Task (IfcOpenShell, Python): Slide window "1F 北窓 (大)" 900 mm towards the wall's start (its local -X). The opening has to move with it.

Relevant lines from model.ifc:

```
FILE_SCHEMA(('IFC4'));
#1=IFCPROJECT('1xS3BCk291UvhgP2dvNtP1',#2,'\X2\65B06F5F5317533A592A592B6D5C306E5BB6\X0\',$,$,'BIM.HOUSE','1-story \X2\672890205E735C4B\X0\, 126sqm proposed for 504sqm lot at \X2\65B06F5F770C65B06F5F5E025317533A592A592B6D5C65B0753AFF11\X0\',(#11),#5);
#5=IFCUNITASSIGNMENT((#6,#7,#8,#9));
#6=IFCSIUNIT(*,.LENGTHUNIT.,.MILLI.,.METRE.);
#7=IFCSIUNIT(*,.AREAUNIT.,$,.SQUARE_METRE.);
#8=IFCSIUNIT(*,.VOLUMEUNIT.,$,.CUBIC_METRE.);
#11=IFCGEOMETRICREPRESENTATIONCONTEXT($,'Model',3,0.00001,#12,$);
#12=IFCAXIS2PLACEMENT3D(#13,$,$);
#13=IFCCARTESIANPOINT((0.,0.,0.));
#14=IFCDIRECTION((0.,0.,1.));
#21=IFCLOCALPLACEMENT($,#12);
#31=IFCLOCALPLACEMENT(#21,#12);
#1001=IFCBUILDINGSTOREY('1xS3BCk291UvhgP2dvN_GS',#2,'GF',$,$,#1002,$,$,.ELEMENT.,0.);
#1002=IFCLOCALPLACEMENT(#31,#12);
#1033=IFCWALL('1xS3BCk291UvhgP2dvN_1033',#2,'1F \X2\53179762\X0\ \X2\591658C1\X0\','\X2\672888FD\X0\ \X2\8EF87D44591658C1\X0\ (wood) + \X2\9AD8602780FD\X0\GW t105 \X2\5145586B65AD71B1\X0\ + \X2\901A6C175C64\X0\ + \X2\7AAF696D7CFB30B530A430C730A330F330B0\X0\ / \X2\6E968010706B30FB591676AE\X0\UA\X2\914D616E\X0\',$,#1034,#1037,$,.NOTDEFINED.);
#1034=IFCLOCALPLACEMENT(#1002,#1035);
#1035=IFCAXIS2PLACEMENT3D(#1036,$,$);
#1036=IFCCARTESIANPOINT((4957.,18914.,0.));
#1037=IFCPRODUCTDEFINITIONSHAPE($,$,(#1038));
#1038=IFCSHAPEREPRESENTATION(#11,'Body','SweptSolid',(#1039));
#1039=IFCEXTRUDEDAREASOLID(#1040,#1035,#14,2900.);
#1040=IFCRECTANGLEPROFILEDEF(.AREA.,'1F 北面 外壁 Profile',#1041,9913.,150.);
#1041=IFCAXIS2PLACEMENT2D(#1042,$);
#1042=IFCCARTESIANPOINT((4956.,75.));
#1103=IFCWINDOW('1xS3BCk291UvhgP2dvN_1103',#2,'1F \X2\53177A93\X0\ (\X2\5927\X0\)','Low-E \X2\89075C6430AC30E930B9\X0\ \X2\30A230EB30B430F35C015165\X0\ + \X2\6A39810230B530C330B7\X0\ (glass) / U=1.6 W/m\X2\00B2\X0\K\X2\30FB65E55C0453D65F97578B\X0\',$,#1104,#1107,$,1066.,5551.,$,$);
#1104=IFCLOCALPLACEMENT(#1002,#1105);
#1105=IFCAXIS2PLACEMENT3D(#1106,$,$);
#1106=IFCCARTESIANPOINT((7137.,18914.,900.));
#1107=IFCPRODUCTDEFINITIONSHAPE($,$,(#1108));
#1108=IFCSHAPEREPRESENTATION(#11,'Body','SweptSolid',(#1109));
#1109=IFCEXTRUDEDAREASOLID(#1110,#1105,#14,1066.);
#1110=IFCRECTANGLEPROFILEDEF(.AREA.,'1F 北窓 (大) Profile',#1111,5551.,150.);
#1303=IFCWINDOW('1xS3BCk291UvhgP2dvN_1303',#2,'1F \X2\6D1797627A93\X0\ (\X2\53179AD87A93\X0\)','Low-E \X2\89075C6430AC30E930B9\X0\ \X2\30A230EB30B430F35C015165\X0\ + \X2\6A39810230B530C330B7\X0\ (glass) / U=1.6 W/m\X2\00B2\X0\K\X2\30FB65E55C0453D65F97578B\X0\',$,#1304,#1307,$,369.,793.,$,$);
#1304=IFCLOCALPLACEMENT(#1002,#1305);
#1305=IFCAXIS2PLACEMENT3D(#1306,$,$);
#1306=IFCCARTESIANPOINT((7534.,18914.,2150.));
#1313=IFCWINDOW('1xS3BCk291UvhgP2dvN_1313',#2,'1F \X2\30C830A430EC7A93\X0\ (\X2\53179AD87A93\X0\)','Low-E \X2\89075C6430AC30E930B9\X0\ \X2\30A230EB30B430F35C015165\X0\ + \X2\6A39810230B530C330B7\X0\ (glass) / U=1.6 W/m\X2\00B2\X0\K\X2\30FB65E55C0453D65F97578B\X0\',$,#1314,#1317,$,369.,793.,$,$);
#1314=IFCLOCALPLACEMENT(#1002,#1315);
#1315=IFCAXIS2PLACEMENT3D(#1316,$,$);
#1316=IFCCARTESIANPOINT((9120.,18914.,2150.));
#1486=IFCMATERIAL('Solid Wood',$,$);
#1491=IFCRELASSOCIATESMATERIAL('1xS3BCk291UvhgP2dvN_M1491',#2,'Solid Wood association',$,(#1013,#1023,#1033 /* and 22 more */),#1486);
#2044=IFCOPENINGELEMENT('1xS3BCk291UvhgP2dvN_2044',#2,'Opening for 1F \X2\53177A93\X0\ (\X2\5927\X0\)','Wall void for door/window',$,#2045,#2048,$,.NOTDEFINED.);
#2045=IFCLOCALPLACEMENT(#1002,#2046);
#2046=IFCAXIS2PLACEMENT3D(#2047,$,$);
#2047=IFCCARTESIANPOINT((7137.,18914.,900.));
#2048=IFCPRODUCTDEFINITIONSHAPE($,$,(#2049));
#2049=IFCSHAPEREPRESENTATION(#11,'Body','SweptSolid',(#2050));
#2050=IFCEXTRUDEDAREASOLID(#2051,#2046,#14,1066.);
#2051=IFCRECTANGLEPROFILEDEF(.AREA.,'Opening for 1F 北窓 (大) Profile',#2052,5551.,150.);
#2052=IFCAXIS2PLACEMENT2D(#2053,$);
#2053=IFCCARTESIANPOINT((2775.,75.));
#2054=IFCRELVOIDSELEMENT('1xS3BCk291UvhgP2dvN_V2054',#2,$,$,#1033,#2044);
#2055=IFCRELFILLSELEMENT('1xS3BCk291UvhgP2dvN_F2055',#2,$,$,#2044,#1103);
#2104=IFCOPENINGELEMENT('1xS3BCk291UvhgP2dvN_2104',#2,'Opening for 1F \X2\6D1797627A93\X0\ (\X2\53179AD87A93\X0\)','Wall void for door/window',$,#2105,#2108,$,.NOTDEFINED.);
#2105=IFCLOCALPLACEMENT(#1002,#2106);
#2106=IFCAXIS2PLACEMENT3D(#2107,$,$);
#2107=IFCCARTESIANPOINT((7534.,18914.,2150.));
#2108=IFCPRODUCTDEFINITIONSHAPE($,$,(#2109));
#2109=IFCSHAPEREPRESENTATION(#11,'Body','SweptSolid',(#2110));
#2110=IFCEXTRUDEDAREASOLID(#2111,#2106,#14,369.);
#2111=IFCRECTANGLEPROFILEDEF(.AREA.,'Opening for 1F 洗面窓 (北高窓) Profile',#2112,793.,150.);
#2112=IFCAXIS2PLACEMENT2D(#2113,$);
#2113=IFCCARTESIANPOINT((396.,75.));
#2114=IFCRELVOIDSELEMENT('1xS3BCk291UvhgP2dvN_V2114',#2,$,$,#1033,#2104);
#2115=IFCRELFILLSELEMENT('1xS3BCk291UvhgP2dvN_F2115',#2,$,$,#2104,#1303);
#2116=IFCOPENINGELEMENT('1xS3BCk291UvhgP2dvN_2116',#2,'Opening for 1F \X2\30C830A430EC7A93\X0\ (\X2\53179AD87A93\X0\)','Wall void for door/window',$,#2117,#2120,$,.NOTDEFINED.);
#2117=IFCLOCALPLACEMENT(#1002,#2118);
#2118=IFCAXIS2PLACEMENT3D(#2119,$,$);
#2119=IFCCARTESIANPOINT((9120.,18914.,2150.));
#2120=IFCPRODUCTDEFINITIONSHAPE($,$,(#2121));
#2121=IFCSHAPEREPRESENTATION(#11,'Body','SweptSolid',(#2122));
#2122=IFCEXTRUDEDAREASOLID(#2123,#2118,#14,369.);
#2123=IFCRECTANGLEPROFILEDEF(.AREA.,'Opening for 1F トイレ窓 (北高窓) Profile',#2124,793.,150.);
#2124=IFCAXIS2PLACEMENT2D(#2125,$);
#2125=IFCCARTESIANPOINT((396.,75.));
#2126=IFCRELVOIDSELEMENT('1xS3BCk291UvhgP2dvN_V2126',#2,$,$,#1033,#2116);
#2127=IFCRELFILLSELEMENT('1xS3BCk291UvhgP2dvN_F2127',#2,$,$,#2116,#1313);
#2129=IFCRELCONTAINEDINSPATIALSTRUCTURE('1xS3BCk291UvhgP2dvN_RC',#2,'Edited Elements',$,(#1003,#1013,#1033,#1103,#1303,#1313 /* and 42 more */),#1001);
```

```python
import ifcopenshell
import ifcopenshell.api.geometry
import ifcopenshell.util.placement
import ifcopenshell.util.unit

model = ifcopenshell.open("model.ifc")
unit_scale = ifcopenshell.util.unit.calculate_unit_scale(model)

window = model.by_id(1103)
opening = window.FillsVoids[0].RelatingOpeningElement
wall = opening.VoidsElements[0].RelatingBuildingElement

wall_matrix = ifcopenshell.util.placement.get_local_placement(wall.ObjectPlacement)
shift = wall_matrix[:3, 0] * -0.9 / unit_scale
before = ifcopenshell.util.placement.get_local_placement(window.ObjectPlacement)[:3, 3].copy()

# The window is not placed relative to its opening, so move both.
for product in (opening, window):
    matrix = ifcopenshell.util.placement.get_local_placement(product.ObjectPlacement)
    matrix[:3, 3] += shift
    ifcopenshell.api.geometry.edit_object_placement(model, product=product, matrix=matrix, is_si=False)

after = ifcopenshell.util.placement.get_local_placement(window.ObjectPlacement)[:3, 3]
print("window moved by", (after - before).round(3) + 0.0)

model.write("model_rev.ifc")
```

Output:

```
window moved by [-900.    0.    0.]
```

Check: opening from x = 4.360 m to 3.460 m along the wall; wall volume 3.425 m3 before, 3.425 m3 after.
